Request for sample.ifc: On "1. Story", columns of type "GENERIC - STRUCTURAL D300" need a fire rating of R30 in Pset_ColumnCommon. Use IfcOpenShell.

First a look at what the model holds.

```python
import ifcopenshell
import ifcopenshell.util.element

model = ifcopenshell.open("sample.ifc")
print(model.schema)
storey = next(s for s in model.by_type("IfcBuildingStorey") if s.Name == "1. Story")
columns = [e for e in ifcopenshell.util.element.get_decomposition(storey) if e.is_a("IfcColumn")]
seen = {}
for e in columns:
    element_type = ifcopenshell.util.element.get_type(e)
    key = (element_type.Name if element_type != e and element_type else None, ifcopenshell.util.element.get_pset(e, "Pset_ColumnCommon", "FireRating"))
    seen[key] = seen.get(key, 0) + 1
for (name, value), count in sorted(seen.items(), key=str):
    print(count, "x", name, "|", value)
```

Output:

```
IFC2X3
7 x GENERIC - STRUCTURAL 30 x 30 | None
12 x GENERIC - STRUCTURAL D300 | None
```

```python
import ifcopenshell
import ifcopenshell.api.pset
import ifcopenshell.util.element

model = ifcopenshell.open("sample.ifc")

storey = next(s for s in model.by_type("IfcBuildingStorey") if s.Name == "1. Story")
columns = [e for e in ifcopenshell.util.element.get_decomposition(storey) if e.is_a("IfcColumn")]

count = 0
for e in columns:
    element_type = ifcopenshell.util.element.get_type(e)
    if element_type in (None, e) or element_type.Name != "GENERIC - STRUCTURAL D300":
        continue
    # add_pset returns the element's existing set when there is one.
    pset = ifcopenshell.api.pset.add_pset(model, product=e, name="Pset_ColumnCommon")
    ifcopenshell.api.pset.edit_pset(model, pset=pset, properties={"FireRating": "R30"})
    count += 1

print(count, "columns updated")

model.write("sample-out.ifc")
```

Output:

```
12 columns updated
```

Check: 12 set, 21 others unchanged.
